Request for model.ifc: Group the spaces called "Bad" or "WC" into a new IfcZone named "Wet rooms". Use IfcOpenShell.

First a look at what the model holds.

```python
import ifcopenshell

model = ifcopenshell.open("model.ifc")
print(model.schema)
seen = {}
for space in model.by_type("IfcSpace"):
    seen[space.LongName] = seen.get(space.LongName, 0) + 1
for name, count in sorted(seen.items(), key=str):
    print(count, "x", name)
print("zones:", [z.Name for z in model.by_type("IfcZone")][:20])
```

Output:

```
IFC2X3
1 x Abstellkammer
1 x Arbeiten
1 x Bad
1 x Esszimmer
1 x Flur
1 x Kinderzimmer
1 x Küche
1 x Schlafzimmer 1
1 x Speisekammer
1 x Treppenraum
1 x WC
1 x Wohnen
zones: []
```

```python
import ifcopenshell
import ifcopenshell.api.group
import ifcopenshell.api.root

model = ifcopenshell.open("model.ifc")

names = {"Bad", "WC"}
spaces = [s for s in model.by_type("IfcSpace") if s.LongName in names]

zone = ifcopenshell.api.root.create_entity(model, ifc_class="IfcZone", name="Wet rooms")
ifcopenshell.api.group.assign_group(model, products=spaces, group=zone)
print(len(spaces), "spaces in", zone.Name)

model.write("model_v2.ifc")
```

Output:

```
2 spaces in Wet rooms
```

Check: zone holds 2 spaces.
